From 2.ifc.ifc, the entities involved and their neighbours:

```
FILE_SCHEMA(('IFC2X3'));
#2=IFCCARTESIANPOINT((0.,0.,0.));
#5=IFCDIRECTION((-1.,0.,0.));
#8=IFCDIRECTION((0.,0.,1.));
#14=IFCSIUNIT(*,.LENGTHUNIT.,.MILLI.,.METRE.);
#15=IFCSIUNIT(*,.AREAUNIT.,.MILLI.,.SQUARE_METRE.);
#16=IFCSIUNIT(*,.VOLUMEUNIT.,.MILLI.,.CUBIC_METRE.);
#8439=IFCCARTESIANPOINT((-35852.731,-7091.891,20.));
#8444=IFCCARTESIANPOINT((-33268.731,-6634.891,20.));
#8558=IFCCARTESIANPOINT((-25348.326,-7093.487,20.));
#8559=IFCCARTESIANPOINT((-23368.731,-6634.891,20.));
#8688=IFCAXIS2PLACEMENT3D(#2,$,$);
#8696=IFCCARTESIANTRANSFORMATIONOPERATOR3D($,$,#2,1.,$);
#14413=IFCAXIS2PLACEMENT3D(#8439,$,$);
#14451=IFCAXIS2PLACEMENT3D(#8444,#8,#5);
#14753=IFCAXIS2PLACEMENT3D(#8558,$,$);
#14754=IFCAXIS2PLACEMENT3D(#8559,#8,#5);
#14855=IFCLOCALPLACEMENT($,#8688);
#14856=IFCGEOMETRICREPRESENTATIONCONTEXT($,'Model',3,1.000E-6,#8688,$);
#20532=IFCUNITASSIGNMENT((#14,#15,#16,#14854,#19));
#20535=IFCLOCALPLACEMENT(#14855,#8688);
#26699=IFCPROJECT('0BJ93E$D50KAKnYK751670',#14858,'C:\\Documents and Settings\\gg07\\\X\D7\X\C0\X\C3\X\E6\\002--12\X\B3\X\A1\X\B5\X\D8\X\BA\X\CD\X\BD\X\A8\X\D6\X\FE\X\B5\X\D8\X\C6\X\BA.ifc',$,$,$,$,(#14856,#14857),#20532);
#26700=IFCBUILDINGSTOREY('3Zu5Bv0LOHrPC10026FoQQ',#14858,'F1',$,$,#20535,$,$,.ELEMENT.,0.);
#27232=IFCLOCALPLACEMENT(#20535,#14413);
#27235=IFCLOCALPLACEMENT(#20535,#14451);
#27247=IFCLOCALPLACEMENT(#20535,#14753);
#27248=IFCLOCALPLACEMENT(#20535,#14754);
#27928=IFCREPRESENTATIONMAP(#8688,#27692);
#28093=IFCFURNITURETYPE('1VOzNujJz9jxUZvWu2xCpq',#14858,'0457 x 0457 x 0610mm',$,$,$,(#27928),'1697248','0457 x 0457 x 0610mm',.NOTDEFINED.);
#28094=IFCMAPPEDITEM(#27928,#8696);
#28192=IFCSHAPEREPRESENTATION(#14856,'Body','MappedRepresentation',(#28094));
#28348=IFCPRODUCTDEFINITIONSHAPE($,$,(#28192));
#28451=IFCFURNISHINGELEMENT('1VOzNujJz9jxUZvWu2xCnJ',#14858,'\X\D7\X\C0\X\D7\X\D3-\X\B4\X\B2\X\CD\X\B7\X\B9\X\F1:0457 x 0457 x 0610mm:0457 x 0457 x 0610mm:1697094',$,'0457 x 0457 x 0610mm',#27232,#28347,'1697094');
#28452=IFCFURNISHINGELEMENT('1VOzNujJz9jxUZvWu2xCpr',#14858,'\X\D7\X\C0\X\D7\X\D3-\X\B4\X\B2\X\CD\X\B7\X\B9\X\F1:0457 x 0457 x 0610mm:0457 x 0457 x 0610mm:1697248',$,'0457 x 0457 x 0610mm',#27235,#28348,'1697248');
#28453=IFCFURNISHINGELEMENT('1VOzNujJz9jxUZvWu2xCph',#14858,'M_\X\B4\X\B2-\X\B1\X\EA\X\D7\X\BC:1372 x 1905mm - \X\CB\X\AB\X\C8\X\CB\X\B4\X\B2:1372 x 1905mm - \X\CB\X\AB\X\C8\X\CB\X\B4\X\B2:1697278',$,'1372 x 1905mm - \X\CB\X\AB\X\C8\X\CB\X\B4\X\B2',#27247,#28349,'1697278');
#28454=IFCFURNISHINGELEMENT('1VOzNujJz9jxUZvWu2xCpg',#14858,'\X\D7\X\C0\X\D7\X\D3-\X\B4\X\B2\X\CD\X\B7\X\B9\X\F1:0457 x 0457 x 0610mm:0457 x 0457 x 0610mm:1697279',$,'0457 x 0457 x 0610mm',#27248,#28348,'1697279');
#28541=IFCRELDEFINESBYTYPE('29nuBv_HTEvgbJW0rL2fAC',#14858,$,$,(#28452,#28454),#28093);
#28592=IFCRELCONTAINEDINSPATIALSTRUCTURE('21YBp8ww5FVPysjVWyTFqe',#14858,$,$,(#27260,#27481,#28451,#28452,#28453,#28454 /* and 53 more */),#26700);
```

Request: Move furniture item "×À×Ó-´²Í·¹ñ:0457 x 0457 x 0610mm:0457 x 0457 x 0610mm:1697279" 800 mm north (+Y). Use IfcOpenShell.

```python
import ifcopenshell
import ifcopenshell.api.geometry
import ifcopenshell.util.placement

model = ifcopenshell.open("2.ifc.ifc")

item = model.by_guid("1VOzNujJz9jxUZvWu2xCpg")
matrix = ifcopenshell.util.placement.get_local_placement(item.ObjectPlacement)
matrix[1, 3] += 800.0
ifcopenshell.api.geometry.edit_object_placement(model, product=item, matrix=matrix, is_si=False)

print(ifcopenshell.util.placement.get_local_placement(item.ObjectPlacement).round(3) + 0.0)

model.write("2.ifc_updated.ifc")
```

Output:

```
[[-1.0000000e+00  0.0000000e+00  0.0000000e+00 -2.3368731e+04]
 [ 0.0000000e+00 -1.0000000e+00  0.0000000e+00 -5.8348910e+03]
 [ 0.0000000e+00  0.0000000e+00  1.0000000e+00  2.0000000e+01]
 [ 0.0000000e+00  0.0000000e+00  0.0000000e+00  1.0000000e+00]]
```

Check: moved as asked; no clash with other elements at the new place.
